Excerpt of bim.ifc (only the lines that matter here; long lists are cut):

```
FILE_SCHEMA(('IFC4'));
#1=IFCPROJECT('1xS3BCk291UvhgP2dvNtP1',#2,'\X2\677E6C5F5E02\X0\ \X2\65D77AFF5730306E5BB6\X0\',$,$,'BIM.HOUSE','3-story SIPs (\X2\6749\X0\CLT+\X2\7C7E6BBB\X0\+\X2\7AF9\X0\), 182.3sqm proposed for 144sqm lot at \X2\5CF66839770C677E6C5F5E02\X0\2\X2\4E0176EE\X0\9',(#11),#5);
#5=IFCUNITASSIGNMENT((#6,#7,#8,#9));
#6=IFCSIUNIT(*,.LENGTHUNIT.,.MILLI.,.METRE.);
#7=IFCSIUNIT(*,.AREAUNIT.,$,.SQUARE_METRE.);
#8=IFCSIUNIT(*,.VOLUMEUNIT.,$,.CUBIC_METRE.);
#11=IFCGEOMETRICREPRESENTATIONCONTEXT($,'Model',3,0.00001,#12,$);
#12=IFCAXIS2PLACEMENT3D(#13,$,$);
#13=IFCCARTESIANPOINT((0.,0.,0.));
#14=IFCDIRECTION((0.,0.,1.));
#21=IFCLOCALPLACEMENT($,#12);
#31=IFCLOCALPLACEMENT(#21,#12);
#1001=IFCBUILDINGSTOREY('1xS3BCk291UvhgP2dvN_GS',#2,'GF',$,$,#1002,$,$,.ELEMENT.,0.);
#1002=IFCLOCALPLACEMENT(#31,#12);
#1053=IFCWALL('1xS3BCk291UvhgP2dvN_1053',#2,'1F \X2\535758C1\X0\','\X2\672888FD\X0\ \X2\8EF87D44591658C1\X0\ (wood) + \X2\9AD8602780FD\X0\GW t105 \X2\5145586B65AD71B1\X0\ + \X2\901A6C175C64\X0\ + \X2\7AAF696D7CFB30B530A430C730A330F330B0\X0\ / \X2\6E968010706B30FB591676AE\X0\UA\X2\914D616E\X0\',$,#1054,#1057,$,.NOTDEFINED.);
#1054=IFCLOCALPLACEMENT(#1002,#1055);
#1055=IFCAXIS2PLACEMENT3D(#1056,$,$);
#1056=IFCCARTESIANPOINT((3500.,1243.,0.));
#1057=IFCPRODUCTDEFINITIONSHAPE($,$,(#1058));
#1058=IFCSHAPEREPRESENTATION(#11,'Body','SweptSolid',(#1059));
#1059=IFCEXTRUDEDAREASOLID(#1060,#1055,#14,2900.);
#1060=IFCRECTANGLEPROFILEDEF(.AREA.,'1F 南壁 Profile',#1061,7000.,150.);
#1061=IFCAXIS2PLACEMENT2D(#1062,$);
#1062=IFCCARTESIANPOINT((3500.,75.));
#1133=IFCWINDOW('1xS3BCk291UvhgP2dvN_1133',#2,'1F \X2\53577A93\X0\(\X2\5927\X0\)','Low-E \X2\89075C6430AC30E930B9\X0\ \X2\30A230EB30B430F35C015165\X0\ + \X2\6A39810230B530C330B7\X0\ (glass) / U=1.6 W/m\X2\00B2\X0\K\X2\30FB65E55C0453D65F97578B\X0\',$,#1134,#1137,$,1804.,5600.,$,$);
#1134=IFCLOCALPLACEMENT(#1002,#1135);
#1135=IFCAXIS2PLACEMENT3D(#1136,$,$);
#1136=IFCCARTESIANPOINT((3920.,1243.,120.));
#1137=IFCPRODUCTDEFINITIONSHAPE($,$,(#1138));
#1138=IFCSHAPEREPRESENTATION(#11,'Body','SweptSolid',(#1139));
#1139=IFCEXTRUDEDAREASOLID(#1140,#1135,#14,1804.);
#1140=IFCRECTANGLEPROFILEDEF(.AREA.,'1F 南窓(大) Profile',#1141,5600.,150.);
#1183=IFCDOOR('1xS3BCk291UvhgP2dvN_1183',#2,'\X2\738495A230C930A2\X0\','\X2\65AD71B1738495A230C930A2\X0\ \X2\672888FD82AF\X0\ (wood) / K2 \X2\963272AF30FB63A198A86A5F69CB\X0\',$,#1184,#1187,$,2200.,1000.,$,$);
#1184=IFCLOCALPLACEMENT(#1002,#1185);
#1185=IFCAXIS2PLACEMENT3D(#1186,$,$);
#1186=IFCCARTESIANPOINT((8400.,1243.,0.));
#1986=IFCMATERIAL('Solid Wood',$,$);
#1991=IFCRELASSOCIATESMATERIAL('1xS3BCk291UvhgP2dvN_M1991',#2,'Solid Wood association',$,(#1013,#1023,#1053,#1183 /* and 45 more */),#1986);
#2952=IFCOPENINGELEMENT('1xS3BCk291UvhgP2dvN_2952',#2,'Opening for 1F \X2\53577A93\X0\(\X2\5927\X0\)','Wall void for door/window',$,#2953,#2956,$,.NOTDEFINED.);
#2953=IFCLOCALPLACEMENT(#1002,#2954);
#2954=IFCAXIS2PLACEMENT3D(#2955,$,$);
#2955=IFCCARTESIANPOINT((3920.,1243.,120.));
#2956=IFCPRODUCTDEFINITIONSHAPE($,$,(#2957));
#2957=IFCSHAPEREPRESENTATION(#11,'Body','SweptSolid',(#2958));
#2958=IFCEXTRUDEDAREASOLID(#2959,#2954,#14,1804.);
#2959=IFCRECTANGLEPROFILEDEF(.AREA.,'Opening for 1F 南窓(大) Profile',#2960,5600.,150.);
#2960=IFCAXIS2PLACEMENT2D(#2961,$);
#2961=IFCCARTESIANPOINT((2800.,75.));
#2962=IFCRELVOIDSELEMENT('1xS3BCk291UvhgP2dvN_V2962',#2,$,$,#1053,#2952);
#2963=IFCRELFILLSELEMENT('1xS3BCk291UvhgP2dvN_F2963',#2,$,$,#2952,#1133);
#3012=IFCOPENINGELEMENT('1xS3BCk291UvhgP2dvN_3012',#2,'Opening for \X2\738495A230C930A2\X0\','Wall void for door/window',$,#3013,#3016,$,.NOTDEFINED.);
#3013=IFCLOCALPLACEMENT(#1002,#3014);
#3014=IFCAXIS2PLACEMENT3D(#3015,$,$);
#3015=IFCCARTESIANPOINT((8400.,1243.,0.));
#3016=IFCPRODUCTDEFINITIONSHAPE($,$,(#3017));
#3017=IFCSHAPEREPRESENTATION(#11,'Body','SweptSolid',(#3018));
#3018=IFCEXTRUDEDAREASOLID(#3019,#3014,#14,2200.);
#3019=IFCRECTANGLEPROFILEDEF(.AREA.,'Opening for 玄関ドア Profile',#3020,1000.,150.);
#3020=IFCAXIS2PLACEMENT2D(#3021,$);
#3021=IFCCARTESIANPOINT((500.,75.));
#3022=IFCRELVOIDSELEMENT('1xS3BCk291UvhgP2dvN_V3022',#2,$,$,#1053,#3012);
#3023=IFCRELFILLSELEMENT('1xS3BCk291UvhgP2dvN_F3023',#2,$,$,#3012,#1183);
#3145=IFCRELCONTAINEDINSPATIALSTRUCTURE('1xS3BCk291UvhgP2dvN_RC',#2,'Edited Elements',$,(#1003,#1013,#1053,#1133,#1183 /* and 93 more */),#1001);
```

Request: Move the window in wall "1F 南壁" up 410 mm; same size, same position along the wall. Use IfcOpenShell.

```python
import numpy as np
import ifcopenshell
import ifcopenshell.api.geometry
import ifcopenshell.util.placement
import ifcopenshell.util.unit

model = ifcopenshell.open("bim.ifc")
unit_scale = ifcopenshell.util.unit.calculate_unit_scale(model)

window = model.by_guid("1xS3BCk291UvhgP2dvN_1133")
opening = window.FillsVoids[0].RelatingOpeningElement
dz = 0.41 / unit_scale

shift = np.array([0.0, 0.0, dz])
# The window is not placed relative to its opening, so move both.
for product in (opening, window):
    matrix = ifcopenshell.util.placement.get_local_placement(product.ObjectPlacement)
    matrix[:3, 3] += shift
    ifcopenshell.api.geometry.edit_object_placement(model, product=product, matrix=matrix, is_si=False)

print(f"moved by {dz * unit_scale:+.3f} m")

model.write("bim_edited.ifc")
```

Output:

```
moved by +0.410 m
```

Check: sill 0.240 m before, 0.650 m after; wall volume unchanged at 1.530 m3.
